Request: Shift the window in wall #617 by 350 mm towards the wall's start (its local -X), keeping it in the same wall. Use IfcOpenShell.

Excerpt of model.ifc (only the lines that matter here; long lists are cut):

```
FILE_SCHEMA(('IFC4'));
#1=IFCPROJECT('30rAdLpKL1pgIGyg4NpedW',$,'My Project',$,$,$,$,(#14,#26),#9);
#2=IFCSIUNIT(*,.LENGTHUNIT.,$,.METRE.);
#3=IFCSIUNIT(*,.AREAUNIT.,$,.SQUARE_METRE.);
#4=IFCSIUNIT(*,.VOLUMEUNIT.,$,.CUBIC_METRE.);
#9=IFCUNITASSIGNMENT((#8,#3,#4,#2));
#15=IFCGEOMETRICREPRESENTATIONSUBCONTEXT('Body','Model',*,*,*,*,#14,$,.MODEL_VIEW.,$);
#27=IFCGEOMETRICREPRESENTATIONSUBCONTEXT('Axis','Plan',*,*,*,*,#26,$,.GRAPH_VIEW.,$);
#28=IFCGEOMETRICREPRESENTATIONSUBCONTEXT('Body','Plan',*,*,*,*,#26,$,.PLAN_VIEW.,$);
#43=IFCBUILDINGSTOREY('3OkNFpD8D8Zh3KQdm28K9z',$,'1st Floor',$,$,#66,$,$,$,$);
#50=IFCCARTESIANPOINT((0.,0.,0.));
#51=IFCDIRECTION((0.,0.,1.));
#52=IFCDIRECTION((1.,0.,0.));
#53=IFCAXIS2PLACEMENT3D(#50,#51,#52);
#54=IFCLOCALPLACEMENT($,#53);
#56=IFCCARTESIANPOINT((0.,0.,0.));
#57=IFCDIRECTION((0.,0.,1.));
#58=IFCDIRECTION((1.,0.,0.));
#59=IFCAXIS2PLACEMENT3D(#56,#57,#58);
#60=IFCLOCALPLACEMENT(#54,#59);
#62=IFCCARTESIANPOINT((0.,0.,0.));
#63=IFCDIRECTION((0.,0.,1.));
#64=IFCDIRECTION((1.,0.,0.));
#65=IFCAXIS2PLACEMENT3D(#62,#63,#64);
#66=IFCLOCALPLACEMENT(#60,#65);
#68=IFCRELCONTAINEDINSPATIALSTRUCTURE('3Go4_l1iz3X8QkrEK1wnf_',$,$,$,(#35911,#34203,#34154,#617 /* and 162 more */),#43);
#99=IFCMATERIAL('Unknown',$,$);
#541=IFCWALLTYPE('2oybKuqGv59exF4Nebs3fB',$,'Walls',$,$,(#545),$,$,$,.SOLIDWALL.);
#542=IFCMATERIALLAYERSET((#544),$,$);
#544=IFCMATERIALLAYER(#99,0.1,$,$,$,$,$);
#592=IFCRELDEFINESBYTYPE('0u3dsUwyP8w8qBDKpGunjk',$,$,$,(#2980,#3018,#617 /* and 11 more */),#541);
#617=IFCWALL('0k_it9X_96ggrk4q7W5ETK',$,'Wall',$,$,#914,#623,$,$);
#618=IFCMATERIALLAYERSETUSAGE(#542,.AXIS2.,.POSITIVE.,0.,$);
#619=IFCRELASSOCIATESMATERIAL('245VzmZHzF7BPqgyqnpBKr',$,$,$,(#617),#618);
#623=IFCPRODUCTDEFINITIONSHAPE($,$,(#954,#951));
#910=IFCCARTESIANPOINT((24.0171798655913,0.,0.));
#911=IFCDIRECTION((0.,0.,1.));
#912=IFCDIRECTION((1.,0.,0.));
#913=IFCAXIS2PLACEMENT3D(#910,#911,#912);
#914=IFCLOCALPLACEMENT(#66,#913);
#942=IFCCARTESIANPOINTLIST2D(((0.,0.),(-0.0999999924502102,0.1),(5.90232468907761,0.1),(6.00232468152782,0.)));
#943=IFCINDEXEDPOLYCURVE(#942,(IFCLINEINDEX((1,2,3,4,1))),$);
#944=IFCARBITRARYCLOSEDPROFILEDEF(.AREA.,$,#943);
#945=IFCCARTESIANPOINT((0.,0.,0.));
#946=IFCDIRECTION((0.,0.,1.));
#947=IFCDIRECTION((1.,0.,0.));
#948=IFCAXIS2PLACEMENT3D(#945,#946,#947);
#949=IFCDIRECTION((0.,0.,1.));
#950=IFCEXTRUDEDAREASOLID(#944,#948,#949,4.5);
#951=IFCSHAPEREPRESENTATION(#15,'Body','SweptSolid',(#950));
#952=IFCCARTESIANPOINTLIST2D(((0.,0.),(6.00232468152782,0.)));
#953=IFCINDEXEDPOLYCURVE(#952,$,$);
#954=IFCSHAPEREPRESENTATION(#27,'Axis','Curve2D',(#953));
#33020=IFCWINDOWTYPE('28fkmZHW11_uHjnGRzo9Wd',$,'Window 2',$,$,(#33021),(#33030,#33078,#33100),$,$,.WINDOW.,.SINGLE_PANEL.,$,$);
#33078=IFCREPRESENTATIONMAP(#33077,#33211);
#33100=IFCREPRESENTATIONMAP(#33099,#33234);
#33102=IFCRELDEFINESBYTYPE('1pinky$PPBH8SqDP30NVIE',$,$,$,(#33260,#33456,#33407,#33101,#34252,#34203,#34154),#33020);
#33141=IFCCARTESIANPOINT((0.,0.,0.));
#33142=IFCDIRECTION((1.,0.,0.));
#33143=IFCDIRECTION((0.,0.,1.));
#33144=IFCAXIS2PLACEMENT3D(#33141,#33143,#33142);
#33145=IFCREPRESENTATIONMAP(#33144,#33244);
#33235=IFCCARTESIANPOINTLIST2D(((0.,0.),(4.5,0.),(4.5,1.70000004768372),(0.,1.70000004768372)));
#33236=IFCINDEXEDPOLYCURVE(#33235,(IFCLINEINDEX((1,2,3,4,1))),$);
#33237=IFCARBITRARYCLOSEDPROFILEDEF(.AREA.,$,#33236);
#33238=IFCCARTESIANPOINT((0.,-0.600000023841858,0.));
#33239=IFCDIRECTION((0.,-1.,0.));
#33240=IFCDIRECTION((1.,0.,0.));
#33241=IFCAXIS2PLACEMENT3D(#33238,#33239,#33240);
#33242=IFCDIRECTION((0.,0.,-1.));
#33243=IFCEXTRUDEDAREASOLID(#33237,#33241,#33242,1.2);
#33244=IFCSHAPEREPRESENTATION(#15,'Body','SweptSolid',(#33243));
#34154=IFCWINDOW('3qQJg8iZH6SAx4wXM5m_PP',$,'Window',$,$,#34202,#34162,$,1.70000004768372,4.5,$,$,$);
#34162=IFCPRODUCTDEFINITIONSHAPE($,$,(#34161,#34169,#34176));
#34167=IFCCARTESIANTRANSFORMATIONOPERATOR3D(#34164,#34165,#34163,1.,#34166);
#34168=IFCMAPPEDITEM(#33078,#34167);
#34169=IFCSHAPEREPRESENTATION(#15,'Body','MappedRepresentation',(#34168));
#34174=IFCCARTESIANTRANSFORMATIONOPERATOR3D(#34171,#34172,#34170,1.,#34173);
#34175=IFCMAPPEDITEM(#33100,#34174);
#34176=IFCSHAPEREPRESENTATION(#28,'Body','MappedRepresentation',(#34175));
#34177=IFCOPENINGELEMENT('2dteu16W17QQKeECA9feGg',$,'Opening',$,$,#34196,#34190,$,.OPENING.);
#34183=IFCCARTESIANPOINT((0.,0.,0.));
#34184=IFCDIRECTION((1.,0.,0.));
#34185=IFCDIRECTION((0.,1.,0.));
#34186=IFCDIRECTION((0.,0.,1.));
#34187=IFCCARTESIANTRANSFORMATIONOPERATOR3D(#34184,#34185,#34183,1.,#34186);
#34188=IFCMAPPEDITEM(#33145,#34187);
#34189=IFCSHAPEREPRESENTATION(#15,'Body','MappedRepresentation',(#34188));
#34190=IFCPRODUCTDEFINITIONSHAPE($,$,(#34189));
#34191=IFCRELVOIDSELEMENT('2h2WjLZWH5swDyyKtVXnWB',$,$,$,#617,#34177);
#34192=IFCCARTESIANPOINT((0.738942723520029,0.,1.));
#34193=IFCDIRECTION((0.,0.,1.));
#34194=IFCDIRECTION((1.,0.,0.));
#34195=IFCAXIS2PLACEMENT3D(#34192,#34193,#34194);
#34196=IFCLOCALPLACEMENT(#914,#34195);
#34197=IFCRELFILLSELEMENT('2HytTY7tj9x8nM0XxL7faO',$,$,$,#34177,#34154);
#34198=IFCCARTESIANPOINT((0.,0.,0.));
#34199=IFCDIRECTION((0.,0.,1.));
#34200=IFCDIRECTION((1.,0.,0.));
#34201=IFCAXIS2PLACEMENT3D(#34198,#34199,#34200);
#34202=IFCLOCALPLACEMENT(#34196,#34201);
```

```python
import ifcopenshell
import ifcopenshell.api.geometry
import ifcopenshell.util.placement
import ifcopenshell.util.unit

model = ifcopenshell.open("model.ifc")
unit_scale = ifcopenshell.util.unit.calculate_unit_scale(model)

window = model.by_guid("3qQJg8iZH6SAx4wXM5m_PP")
opening = window.FillsVoids[0].RelatingOpeningElement
wall = opening.VoidsElements[0].RelatingBuildingElement

wall_matrix = ifcopenshell.util.placement.get_local_placement(wall.ObjectPlacement)
shift = wall_matrix[:3, 0] * -0.35 / unit_scale
before = ifcopenshell.util.placement.get_local_placement(window.ObjectPlacement)[:3, 3].copy()

# The window is placed relative to its opening, so it follows when the opening moves.
matrix = ifcopenshell.util.placement.get_local_placement(opening.ObjectPlacement)
matrix[:3, 3] += shift
ifcopenshell.api.geometry.edit_object_placement(
    model, product=opening, matrix=matrix, is_si=False, should_transform_children=True
)

after = ifcopenshell.util.placement.get_local_placement(window.ObjectPlacement)[:3, 3]
print("window moved by", (after - before).round(3) + 0.0)

model.write("model_v2.ifc")
```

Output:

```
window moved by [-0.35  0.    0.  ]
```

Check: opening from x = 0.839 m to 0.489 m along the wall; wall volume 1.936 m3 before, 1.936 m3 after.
